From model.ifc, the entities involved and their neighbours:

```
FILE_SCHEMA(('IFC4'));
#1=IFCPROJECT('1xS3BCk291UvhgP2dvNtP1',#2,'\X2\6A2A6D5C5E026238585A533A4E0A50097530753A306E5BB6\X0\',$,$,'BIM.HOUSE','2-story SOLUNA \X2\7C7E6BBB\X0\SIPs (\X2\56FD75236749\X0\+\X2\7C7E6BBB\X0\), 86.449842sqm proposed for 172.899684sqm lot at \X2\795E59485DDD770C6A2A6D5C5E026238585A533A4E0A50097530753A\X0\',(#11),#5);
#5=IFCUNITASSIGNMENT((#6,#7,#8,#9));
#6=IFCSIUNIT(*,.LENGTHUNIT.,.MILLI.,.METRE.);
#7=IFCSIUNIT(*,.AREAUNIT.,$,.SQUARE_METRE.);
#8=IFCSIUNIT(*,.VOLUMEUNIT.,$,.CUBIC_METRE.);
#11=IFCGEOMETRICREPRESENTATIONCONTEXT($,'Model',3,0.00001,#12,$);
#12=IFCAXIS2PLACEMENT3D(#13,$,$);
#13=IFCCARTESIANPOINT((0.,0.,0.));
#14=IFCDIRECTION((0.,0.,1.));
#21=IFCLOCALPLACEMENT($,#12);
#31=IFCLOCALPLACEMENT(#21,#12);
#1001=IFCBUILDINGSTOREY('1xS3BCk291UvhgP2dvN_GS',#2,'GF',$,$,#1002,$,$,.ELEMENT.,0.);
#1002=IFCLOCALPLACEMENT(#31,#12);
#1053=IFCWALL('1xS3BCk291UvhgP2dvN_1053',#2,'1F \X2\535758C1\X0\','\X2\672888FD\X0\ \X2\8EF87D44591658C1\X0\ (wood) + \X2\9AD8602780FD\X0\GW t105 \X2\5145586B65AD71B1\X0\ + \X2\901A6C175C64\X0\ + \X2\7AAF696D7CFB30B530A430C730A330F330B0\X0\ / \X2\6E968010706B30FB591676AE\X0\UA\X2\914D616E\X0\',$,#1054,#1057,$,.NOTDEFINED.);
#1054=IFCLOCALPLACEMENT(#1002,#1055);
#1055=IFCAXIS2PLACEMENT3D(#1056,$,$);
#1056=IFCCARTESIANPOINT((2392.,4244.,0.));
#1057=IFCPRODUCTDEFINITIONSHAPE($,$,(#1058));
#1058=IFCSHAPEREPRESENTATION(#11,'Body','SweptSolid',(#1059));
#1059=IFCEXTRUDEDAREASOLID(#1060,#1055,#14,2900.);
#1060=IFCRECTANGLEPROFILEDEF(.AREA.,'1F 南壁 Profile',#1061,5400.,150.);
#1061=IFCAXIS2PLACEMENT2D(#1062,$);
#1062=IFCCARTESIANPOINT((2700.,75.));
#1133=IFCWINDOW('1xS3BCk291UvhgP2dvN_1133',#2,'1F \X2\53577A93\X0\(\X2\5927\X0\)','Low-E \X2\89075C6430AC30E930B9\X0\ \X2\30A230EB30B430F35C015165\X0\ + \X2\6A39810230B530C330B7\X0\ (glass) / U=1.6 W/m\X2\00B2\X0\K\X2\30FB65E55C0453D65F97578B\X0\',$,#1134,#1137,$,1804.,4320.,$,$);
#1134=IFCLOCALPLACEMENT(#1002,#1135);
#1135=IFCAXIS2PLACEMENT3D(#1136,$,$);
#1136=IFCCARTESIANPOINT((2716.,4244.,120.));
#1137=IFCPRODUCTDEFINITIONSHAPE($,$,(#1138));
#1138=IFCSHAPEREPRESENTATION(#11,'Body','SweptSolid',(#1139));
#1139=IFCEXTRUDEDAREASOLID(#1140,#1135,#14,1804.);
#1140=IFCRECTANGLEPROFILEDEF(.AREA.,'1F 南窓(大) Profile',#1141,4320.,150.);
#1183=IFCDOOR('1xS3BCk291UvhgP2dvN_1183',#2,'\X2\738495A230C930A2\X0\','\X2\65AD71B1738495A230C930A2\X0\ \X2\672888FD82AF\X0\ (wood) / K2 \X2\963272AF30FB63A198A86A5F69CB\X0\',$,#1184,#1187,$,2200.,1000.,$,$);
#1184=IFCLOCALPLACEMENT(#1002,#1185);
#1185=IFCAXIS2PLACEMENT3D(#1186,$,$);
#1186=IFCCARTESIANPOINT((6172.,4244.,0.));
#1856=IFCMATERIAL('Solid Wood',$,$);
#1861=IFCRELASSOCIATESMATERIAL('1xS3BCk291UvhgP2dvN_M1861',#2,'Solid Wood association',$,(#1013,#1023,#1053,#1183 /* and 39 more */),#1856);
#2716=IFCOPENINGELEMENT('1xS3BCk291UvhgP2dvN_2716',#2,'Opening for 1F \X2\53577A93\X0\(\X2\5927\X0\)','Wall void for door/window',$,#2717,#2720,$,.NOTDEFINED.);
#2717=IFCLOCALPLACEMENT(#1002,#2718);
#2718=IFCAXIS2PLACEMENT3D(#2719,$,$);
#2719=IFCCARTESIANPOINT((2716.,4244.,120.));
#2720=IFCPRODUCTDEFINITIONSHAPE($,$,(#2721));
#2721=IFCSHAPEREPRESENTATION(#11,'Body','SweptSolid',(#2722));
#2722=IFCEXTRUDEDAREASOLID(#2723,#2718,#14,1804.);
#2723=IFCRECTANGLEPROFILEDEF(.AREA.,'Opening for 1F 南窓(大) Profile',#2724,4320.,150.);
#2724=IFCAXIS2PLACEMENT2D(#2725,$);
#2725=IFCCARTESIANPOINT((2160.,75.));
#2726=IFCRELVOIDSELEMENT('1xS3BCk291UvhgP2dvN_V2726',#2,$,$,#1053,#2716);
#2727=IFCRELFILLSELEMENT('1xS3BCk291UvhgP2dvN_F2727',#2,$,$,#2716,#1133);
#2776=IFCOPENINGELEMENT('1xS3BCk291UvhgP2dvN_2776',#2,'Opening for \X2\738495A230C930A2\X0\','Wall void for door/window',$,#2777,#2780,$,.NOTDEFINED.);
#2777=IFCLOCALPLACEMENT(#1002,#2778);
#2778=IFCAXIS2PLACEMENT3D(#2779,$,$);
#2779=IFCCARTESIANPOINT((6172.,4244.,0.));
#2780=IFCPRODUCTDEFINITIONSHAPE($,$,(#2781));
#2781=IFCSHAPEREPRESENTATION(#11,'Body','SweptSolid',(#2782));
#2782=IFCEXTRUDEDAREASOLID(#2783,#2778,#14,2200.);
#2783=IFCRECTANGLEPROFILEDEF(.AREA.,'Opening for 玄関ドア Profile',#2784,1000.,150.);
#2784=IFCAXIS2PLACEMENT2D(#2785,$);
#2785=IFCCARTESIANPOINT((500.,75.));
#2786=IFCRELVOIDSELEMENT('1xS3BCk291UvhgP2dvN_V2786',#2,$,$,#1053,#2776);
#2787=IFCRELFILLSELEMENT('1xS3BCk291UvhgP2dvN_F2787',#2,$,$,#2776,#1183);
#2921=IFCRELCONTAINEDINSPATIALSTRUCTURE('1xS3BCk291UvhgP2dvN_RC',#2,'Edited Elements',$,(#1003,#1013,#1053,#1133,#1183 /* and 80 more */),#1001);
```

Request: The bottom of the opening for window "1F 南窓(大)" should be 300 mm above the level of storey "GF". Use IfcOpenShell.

```python
import numpy as np
import ifcopenshell
import ifcopenshell.api.geometry
import ifcopenshell.geom
import ifcopenshell.util.element
import ifcopenshell.util.placement
import ifcopenshell.util.shape
import ifcopenshell.util.unit

model = ifcopenshell.open("model.ifc")
unit_scale = ifcopenshell.util.unit.calculate_unit_scale(model)

window = model.by_guid("1xS3BCk291UvhgP2dvN_1133")
opening = window.FillsVoids[0].RelatingOpeningElement
storey = ifcopenshell.util.element.get_container(window, ifc_class="IfcBuildingStorey")
level = ifcopenshell.util.placement.get_local_placement(storey.ObjectPlacement)[2, 3]

# The opening's origin need not be at the sill, so measure its lowest point.
shape = ifcopenshell.geom.create_shape(ifcopenshell.geom.settings(), opening)
bottom = ifcopenshell.util.shape.get_shape_bottom_elevation(shape, shape.geometry) / unit_scale
dz = level + 300.0 - bottom

shift = np.array([0.0, 0.0, dz])
# The window is not placed relative to its opening, so move both.
for product in (opening, window):
    matrix = ifcopenshell.util.placement.get_local_placement(product.ObjectPlacement)
    matrix[:3, 3] += shift
    ifcopenshell.api.geometry.edit_object_placement(model, product=product, matrix=matrix, is_si=False)

print(f"moved by {dz * unit_scale:+.3f} m")

model.write("model_updated.ifc")
```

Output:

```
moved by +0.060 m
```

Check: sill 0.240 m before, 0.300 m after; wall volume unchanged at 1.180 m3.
